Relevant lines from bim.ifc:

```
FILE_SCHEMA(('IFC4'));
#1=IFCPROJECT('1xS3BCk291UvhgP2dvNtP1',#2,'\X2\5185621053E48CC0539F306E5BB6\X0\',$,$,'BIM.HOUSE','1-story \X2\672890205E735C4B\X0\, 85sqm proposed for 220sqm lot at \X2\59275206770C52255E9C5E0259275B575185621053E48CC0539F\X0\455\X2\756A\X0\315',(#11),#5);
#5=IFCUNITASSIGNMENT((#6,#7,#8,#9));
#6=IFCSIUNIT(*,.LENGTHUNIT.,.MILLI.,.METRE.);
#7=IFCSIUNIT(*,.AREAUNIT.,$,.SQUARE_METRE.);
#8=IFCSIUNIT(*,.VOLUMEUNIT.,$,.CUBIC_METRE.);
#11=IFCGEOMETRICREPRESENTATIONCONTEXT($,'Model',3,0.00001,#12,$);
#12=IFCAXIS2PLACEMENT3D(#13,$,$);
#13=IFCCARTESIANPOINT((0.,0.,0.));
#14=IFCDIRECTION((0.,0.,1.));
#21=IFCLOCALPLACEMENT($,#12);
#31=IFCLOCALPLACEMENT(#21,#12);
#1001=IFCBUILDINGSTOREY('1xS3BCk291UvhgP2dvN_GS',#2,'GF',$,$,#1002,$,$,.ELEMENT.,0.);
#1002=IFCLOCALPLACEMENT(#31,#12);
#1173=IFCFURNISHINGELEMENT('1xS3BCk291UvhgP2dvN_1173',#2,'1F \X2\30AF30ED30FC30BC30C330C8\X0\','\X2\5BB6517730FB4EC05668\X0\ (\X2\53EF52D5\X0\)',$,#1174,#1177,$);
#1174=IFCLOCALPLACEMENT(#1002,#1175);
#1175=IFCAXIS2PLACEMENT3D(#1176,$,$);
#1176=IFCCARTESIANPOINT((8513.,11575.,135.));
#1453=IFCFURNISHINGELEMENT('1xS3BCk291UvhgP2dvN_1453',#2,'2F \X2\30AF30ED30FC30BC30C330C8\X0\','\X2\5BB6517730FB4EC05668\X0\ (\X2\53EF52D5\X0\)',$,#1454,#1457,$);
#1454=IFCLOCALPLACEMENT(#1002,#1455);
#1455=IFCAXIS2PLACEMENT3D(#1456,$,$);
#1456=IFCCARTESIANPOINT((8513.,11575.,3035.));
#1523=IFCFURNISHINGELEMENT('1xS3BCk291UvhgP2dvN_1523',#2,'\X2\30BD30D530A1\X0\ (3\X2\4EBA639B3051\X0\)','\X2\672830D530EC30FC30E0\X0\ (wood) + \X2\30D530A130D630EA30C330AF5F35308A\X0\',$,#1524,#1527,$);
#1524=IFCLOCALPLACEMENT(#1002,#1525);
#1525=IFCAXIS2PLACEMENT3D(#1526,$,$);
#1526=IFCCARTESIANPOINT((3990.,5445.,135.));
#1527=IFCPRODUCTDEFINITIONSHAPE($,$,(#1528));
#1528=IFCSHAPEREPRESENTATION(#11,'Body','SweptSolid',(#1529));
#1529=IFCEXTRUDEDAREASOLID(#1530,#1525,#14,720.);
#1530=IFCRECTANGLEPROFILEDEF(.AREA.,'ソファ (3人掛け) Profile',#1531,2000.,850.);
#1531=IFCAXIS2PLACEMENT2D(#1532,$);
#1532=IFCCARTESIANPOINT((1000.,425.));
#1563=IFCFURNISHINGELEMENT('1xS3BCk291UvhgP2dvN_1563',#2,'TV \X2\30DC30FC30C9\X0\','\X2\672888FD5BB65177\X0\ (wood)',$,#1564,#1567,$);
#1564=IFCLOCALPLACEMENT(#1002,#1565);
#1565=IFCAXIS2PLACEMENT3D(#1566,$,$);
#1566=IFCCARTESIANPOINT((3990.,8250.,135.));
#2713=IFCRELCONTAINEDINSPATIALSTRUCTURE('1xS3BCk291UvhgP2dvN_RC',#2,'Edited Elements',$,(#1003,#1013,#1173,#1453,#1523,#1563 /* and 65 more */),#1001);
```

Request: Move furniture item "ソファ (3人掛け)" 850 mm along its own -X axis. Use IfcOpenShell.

```python
import ifcopenshell
import ifcopenshell.api.geometry
import ifcopenshell.util.placement

model = ifcopenshell.open("bim.ifc")

item = model.by_id(1523)
matrix = ifcopenshell.util.placement.get_local_placement(item.ObjectPlacement)
matrix[:3, 3] -= matrix[:3, 0] * 850.0
ifcopenshell.api.geometry.edit_object_placement(model, product=item, matrix=matrix, is_si=False)

print(ifcopenshell.util.placement.get_local_placement(item.ObjectPlacement).round(3) + 0.0)

model.write("bim_edited.ifc")
```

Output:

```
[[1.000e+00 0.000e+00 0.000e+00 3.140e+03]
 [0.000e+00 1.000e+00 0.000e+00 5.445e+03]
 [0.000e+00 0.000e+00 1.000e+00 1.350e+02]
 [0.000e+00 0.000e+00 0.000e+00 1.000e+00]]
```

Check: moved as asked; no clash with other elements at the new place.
